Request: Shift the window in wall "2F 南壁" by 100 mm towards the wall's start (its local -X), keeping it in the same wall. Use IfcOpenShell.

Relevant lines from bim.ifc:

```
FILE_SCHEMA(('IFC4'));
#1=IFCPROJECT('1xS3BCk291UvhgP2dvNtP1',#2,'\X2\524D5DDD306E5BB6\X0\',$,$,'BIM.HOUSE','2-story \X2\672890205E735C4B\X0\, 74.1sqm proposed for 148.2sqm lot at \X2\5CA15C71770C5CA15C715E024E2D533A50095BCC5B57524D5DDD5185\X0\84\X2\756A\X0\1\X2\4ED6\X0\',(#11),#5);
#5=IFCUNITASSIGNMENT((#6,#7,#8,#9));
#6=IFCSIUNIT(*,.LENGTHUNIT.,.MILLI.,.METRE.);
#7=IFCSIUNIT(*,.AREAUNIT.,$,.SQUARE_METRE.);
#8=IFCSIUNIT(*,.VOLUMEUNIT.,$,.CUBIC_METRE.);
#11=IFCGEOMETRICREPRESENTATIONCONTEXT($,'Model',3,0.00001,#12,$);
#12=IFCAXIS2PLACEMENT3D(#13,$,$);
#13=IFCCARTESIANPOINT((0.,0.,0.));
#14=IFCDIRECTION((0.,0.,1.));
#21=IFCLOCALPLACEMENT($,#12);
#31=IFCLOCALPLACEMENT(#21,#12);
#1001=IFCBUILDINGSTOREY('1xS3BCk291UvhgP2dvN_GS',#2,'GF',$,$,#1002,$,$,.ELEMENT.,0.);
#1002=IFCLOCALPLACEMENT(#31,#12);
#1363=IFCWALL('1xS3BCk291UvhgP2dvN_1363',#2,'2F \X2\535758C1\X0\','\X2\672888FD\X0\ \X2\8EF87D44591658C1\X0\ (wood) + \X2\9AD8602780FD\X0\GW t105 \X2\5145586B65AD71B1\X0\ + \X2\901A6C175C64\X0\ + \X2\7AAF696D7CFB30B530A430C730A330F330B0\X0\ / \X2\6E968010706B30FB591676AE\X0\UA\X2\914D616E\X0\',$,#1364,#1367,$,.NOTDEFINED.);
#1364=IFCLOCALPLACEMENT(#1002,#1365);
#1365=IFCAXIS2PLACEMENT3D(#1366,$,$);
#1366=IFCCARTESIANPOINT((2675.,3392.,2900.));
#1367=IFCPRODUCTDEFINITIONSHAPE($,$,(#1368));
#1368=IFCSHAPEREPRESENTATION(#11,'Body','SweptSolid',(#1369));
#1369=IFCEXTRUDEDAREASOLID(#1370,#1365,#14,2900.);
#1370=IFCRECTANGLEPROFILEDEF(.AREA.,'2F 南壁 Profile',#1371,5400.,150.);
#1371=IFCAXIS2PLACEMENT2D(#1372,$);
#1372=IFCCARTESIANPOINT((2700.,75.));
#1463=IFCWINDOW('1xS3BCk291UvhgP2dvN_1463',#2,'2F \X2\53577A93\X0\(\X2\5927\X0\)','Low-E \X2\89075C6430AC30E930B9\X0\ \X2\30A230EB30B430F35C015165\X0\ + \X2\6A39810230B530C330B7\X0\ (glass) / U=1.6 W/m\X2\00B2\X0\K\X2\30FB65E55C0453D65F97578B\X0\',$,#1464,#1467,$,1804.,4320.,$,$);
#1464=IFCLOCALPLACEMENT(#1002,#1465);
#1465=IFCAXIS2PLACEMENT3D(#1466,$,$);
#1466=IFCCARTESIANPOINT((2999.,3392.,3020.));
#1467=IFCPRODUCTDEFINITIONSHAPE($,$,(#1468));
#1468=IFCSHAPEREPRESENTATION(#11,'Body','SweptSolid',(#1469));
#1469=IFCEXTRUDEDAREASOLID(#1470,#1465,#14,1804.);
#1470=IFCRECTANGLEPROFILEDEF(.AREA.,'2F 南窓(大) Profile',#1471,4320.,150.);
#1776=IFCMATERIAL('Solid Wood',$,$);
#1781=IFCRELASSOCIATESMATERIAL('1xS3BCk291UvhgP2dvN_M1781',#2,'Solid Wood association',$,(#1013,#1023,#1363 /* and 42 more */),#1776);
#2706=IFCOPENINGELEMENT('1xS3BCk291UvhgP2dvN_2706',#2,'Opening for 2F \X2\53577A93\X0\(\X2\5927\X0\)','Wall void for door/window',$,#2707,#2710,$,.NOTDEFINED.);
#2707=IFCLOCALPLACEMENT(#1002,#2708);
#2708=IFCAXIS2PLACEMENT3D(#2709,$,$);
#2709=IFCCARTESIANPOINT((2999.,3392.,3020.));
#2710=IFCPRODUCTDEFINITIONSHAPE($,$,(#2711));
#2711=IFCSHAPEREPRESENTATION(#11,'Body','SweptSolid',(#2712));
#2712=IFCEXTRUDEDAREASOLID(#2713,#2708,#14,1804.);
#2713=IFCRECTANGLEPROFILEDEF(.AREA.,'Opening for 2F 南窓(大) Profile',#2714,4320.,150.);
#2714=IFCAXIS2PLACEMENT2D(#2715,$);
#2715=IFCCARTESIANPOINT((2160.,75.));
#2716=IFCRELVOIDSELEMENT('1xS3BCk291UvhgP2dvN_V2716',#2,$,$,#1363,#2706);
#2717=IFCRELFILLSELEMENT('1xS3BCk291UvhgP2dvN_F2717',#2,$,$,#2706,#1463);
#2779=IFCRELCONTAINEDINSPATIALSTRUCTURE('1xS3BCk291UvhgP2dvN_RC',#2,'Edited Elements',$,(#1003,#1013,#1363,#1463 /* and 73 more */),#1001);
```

```python
import ifcopenshell
import ifcopenshell.api.geometry
import ifcopenshell.util.placement
import ifcopenshell.util.unit

model = ifcopenshell.open("bim.ifc")
unit_scale = ifcopenshell.util.unit.calculate_unit_scale(model)

window = model.by_guid("1xS3BCk291UvhgP2dvN_1463")
opening = window.FillsVoids[0].RelatingOpeningElement
wall = opening.VoidsElements[0].RelatingBuildingElement

wall_matrix = ifcopenshell.util.placement.get_local_placement(wall.ObjectPlacement)
shift = wall_matrix[:3, 0] * -0.1 / unit_scale
before = ifcopenshell.util.placement.get_local_placement(window.ObjectPlacement)[:3, 3].copy()

# The window is not placed relative to its opening, so move both.
for product in (opening, window):
    matrix = ifcopenshell.util.placement.get_local_placement(product.ObjectPlacement)
    matrix[:3, 3] += shift
    ifcopenshell.api.geometry.edit_object_placement(model, product=product, matrix=matrix, is_si=False)

after = ifcopenshell.util.placement.get_local_placement(window.ObjectPlacement)[:3, 3]
print("window moved by", (after - before).round(3) + 0.0)

model.write("bim_updated.ifc")
```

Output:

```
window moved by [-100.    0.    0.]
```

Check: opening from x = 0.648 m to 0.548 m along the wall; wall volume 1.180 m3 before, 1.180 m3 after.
